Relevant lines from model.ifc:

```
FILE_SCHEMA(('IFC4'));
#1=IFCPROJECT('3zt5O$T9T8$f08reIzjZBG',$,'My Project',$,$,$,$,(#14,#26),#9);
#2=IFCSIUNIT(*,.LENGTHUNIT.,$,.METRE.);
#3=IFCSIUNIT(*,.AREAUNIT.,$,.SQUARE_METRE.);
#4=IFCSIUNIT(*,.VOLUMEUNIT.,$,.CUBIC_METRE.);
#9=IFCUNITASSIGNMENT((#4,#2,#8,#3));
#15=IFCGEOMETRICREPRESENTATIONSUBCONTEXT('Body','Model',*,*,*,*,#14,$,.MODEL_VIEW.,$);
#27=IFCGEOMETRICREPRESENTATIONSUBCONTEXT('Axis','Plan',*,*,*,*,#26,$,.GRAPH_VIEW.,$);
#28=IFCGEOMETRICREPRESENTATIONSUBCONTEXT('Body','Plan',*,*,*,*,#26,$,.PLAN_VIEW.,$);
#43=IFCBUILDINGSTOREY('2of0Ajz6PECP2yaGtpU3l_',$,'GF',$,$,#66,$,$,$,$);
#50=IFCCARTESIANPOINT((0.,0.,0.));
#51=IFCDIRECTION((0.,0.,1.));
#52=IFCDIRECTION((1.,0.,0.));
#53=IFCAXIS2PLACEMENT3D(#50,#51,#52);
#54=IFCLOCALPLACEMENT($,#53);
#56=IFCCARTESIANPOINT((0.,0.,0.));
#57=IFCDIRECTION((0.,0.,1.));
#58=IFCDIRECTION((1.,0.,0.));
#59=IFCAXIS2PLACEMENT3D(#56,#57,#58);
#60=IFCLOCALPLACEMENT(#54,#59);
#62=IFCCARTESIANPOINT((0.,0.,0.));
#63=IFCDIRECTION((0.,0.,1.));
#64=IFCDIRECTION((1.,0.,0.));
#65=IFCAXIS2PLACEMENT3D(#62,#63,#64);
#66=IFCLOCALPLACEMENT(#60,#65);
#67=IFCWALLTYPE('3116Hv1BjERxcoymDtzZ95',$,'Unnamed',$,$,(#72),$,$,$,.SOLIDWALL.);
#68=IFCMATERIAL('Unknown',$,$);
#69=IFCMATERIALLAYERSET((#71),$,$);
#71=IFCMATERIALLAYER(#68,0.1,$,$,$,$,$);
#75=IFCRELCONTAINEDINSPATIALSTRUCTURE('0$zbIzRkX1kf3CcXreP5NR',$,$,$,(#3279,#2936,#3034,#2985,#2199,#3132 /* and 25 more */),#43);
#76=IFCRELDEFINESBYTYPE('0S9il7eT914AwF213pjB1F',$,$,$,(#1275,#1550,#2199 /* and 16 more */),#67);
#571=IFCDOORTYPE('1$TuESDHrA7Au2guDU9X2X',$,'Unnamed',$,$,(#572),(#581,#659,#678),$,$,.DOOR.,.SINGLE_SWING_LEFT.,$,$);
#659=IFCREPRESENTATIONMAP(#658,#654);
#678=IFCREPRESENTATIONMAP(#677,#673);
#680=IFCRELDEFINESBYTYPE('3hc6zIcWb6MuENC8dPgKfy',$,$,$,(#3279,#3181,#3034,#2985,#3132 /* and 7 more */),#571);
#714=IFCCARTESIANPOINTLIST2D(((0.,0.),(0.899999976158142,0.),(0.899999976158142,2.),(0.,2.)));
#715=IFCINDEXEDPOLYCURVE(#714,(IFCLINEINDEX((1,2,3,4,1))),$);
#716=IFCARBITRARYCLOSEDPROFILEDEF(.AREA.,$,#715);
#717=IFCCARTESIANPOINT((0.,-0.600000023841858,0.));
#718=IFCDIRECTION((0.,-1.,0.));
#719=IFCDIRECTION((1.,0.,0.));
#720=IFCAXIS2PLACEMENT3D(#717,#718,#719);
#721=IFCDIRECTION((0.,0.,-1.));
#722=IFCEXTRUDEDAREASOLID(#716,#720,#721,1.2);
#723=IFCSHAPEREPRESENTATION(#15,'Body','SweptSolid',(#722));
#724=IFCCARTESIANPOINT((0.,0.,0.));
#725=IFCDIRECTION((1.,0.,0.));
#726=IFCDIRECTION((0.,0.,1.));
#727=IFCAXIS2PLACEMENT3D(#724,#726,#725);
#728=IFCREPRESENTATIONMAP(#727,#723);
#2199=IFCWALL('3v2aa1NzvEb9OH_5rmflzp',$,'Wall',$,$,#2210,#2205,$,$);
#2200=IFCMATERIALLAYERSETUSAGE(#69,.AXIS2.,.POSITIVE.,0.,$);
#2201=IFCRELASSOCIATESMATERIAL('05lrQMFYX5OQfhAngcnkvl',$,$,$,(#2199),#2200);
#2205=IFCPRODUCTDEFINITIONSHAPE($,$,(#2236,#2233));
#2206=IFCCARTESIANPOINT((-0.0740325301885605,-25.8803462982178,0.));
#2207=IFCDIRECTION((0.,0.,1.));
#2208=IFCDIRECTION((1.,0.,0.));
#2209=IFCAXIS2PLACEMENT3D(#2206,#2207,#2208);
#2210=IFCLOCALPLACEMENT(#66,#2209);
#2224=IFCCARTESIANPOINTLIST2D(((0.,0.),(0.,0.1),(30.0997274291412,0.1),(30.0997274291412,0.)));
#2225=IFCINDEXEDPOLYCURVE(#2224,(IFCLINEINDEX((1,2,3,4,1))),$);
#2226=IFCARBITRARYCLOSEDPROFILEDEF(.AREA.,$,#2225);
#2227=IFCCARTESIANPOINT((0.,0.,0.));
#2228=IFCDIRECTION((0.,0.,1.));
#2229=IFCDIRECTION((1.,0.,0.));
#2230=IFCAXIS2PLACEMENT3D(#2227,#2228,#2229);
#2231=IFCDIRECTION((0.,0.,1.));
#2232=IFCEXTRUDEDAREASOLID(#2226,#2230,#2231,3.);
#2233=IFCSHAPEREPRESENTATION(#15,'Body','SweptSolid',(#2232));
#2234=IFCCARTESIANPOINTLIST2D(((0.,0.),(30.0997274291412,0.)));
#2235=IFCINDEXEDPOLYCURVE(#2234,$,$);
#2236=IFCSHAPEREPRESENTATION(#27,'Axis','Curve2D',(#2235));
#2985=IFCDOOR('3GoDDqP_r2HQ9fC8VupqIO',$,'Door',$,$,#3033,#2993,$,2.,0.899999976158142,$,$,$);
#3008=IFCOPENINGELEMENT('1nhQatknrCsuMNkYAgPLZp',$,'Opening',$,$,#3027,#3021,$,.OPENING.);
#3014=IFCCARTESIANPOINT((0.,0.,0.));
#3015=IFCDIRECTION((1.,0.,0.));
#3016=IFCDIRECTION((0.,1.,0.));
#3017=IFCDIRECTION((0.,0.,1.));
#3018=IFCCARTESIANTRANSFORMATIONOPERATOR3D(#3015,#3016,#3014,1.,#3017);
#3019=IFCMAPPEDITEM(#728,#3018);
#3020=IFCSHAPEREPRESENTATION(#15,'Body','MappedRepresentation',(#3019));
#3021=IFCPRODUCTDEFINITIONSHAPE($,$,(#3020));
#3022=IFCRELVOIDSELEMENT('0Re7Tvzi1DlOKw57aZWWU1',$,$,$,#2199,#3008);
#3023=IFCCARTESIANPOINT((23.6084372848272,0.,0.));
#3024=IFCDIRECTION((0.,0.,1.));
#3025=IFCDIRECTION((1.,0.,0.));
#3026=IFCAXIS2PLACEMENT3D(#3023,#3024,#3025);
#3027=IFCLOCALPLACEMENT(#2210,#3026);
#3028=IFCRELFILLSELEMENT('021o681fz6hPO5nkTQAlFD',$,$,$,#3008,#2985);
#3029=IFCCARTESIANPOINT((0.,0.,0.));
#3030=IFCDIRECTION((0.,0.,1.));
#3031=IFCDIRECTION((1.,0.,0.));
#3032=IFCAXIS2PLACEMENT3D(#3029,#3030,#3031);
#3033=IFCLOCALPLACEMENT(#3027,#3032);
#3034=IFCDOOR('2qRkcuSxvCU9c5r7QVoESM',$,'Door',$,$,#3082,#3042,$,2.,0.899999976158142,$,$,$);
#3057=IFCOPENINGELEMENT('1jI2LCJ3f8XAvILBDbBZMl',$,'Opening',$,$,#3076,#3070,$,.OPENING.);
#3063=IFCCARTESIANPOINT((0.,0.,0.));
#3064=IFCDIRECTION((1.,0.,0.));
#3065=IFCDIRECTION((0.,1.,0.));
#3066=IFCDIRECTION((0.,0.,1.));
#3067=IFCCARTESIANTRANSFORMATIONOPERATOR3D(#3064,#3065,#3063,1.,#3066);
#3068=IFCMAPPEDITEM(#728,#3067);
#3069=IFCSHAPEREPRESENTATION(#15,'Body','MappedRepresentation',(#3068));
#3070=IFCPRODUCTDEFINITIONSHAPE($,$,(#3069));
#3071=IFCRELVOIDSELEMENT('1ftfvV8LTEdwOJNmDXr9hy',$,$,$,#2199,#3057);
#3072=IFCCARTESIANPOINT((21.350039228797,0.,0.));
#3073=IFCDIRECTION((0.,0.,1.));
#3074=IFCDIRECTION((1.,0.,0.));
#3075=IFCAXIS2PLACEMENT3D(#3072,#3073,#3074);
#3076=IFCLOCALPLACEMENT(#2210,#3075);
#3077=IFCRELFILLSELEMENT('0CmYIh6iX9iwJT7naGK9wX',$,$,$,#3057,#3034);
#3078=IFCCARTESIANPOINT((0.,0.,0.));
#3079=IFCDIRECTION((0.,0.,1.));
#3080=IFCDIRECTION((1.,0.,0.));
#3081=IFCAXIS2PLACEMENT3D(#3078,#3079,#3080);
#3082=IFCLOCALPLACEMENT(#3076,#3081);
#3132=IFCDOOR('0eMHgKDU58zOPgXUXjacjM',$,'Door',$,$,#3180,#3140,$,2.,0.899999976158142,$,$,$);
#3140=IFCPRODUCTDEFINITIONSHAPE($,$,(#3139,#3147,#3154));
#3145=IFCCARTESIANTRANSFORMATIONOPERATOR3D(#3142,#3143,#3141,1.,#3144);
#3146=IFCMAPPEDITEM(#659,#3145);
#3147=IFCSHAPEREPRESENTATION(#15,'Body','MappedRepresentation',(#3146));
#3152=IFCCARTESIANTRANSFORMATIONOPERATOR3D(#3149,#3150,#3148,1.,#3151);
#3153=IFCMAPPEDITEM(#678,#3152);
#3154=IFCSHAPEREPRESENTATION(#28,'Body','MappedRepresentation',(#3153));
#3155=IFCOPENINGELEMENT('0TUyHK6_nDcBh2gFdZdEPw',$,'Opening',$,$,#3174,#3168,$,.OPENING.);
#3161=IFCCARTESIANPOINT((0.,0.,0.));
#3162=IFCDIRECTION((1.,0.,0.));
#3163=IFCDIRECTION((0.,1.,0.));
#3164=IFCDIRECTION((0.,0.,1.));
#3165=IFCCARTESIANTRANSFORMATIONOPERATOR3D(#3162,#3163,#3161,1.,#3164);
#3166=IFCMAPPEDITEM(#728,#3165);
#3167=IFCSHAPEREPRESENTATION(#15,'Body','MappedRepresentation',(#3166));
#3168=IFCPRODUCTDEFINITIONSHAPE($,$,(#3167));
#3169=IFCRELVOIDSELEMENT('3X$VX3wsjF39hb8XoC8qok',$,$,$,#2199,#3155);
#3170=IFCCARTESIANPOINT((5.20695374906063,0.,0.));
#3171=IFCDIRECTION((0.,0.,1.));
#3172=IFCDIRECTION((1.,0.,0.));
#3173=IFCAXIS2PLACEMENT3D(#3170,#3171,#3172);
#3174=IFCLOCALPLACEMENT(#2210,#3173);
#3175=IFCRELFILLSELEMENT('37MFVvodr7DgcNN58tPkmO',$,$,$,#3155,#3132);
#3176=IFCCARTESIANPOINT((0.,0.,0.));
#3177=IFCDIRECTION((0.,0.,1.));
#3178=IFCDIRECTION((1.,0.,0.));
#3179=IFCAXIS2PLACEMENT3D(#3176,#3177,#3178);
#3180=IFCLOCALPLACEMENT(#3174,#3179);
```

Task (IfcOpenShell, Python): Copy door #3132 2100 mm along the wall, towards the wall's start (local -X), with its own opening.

```python
import ifcopenshell
import ifcopenshell.api.feature
import ifcopenshell.api.geometry
import ifcopenshell.api.root
import ifcopenshell.geom
import ifcopenshell.util.element
import ifcopenshell.util.placement
import ifcopenshell.util.shape

model = ifcopenshell.open("model.ifc")
settings = ifcopenshell.geom.settings()


def volume(element):
    """Net volume in cubic metres, openings subtracted."""
    shape = ifcopenshell.geom.create_shape(settings, element)
    return ifcopenshell.util.shape.get_volume(shape.geometry)


door = model.by_id(3132)
opening = door.FillsVoids[0].RelatingOpeningElement
wall = opening.VoidsElements[0].RelatingBuildingElement
before = volume(wall)
shift = ifcopenshell.util.placement.get_local_placement(wall.ObjectPlacement)[:3, 0] * -2.1

# copy_class copies the void relationship, type, container and properties, but no geometry.
new_opening = ifcopenshell.api.root.copy_class(model, product=opening)
new_opening.Representation = ifcopenshell.util.element.copy_deep(
    model, opening.Representation, exclude=["IfcGeometricRepresentationContext", "IfcRepresentationMap"]
)
new_door = ifcopenshell.api.root.copy_class(model, product=door)
new_door.Representation = ifcopenshell.util.element.copy_deep(
    model, door.Representation, exclude=["IfcGeometricRepresentationContext", "IfcRepresentationMap"]
)
ifcopenshell.api.feature.add_filling(model, opening=new_opening, element=new_door)

for old, new in ((opening, new_opening), (door, new_door)):
    matrix = ifcopenshell.util.placement.get_local_placement(old.ObjectPlacement)
    matrix[:3, 3] += shift
    ifcopenshell.api.geometry.edit_object_placement(model, product=new, matrix=matrix, is_si=False)

after = volume(wall)

print(f"wall volume {before:.3f} -> {after:.3f} m3")

model.write("model_updated.ifc")
```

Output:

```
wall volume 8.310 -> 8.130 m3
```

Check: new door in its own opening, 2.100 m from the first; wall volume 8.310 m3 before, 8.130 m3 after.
